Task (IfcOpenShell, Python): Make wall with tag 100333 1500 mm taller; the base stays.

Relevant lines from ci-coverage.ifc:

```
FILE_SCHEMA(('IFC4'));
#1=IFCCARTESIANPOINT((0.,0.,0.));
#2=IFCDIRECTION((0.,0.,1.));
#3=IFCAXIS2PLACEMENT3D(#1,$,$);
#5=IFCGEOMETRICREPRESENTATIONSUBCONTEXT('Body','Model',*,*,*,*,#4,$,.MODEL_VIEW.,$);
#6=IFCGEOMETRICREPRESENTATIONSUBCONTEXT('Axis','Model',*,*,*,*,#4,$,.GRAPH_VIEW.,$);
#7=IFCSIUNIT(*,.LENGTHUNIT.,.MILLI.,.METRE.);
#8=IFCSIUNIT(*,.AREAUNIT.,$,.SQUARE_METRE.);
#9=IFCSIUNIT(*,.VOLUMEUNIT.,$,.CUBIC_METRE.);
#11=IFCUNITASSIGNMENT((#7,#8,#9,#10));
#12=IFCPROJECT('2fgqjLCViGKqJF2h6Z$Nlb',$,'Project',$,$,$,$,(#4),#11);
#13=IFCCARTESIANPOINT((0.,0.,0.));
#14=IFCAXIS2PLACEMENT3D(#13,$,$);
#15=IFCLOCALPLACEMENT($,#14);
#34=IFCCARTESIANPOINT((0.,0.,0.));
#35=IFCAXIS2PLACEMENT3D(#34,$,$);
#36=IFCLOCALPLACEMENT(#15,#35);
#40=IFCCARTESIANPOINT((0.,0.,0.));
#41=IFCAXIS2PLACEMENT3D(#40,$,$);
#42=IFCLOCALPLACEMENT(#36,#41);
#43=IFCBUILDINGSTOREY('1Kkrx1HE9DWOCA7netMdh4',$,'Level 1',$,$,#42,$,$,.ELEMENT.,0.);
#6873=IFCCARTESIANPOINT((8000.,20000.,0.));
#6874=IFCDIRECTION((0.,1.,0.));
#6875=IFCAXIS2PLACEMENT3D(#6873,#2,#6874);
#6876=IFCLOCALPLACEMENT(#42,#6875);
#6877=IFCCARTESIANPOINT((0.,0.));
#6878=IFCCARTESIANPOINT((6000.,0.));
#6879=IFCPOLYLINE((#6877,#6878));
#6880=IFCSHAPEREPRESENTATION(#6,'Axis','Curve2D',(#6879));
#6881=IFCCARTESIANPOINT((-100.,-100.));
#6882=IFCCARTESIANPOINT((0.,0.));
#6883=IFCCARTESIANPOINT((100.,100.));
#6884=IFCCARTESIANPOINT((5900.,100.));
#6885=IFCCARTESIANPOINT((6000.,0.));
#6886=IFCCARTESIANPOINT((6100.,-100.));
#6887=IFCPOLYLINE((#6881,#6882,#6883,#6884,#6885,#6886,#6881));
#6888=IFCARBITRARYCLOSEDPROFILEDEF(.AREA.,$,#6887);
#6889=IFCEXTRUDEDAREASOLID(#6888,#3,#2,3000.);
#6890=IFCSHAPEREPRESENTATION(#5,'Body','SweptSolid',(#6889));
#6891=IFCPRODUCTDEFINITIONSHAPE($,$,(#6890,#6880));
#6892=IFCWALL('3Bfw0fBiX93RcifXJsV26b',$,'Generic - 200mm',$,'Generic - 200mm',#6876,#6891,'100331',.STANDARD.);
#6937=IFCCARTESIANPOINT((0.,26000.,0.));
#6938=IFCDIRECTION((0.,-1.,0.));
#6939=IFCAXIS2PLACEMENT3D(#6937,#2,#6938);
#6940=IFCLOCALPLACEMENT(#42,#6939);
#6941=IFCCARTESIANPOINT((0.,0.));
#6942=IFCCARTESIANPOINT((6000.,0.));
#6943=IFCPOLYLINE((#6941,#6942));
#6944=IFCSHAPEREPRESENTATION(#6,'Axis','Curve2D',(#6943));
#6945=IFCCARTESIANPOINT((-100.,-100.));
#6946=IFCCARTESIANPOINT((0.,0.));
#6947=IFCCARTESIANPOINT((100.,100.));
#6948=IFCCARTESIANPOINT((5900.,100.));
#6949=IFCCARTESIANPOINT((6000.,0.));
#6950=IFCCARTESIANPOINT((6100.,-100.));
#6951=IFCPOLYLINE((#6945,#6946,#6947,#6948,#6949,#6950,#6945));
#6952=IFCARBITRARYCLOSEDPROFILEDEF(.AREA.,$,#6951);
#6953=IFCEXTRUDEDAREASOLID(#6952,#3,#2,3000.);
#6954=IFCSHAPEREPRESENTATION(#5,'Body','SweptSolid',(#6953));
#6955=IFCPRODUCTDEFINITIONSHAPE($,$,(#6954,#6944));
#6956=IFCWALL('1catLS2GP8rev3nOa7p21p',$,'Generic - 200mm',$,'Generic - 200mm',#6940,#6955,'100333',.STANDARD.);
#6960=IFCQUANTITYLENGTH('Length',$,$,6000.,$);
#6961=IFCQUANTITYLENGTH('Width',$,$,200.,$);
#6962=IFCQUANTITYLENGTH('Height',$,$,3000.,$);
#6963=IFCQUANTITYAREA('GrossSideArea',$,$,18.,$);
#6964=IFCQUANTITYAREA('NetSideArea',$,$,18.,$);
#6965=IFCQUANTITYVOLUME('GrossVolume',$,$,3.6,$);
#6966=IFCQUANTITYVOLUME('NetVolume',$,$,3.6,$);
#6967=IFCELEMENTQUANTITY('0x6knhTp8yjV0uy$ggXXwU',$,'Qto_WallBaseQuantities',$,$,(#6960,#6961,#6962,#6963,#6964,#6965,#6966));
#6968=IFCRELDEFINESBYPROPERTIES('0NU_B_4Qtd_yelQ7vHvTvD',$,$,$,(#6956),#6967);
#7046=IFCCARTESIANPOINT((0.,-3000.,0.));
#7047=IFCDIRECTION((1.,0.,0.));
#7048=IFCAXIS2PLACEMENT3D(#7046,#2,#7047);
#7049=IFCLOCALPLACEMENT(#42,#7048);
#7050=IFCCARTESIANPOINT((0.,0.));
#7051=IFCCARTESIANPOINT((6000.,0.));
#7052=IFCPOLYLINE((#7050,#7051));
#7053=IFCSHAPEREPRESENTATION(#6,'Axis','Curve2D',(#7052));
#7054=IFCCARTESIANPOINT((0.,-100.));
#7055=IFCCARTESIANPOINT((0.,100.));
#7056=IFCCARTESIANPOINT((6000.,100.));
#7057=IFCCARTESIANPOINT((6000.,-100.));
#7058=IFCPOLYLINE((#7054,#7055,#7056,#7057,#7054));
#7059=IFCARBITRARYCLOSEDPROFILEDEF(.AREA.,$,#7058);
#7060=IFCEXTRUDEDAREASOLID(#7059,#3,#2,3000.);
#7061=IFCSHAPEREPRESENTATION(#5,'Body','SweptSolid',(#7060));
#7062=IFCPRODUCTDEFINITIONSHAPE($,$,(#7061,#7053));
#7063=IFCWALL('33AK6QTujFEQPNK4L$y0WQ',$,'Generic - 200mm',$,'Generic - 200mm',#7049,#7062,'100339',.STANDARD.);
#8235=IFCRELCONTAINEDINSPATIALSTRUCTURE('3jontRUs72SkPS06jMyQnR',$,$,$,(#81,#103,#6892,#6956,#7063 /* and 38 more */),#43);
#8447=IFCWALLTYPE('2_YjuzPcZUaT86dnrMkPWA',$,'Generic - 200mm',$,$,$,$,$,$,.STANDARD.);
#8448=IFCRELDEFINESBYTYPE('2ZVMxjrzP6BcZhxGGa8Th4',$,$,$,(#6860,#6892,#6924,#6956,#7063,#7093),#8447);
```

```python
import ifcopenshell
import ifcopenshell.api.pset
import ifcopenshell.geom
import ifcopenshell.util.element
import ifcopenshell.util.representation
import ifcopenshell.util.shape
import ifcopenshell.util.unit

model = ifcopenshell.open("ci-coverage.ifc")
unit_scale = ifcopenshell.util.unit.calculate_unit_scale(model)
area_scale = ifcopenshell.util.unit.calculate_unit_scale(model, "AREAUNIT")
volume_scale = ifcopenshell.util.unit.calculate_unit_scale(model, "VOLUMEUNIT")
settings = ifcopenshell.geom.settings()


def volume(element):
    """Net volume in cubic metres, openings subtracted."""
    shape = ifcopenshell.geom.create_shape(settings, element)
    return ifcopenshell.util.shape.get_volume(shape.geometry)


wall = model.by_guid("1catLS2GP8rev3nOa7p21p")
before = volume(wall)

body = ifcopenshell.util.representation.get_representation(wall, "Model", "Body")
solid = body.Items[0]
old_height = solid.Depth
solid.Depth += 1.5 / unit_scale
after = volume(wall)
thickness = 0.2  # wall thickness in metres

# Update the stored height, areas and volumes.
qto = model.by_id(ifcopenshell.util.element.get_pset(wall, "Qto_WallBaseQuantities", should_inherit=False)["id"])
ifcopenshell.api.pset.edit_qto(model, qto=qto, properties={
    "Height": solid.Depth,
    "GrossSideArea": ifcopenshell.util.element.get_pset(wall, "Qto_WallBaseQuantities", "GrossSideArea") * solid.Depth / old_height,
    "NetSideArea": after / thickness / area_scale,
    "GrossVolume": ifcopenshell.util.element.get_pset(wall, "Qto_WallBaseQuantities", "GrossVolume") * solid.Depth / old_height,
    "NetVolume": after / volume_scale,
})

print(f"height {old_height:g} -> {solid.Depth:g}, volume {before:.3f} -> {after:.3f} m3")

model.write("ci-coverage_rev.ifc")
```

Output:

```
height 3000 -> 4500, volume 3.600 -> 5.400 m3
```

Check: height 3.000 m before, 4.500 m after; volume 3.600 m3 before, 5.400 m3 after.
